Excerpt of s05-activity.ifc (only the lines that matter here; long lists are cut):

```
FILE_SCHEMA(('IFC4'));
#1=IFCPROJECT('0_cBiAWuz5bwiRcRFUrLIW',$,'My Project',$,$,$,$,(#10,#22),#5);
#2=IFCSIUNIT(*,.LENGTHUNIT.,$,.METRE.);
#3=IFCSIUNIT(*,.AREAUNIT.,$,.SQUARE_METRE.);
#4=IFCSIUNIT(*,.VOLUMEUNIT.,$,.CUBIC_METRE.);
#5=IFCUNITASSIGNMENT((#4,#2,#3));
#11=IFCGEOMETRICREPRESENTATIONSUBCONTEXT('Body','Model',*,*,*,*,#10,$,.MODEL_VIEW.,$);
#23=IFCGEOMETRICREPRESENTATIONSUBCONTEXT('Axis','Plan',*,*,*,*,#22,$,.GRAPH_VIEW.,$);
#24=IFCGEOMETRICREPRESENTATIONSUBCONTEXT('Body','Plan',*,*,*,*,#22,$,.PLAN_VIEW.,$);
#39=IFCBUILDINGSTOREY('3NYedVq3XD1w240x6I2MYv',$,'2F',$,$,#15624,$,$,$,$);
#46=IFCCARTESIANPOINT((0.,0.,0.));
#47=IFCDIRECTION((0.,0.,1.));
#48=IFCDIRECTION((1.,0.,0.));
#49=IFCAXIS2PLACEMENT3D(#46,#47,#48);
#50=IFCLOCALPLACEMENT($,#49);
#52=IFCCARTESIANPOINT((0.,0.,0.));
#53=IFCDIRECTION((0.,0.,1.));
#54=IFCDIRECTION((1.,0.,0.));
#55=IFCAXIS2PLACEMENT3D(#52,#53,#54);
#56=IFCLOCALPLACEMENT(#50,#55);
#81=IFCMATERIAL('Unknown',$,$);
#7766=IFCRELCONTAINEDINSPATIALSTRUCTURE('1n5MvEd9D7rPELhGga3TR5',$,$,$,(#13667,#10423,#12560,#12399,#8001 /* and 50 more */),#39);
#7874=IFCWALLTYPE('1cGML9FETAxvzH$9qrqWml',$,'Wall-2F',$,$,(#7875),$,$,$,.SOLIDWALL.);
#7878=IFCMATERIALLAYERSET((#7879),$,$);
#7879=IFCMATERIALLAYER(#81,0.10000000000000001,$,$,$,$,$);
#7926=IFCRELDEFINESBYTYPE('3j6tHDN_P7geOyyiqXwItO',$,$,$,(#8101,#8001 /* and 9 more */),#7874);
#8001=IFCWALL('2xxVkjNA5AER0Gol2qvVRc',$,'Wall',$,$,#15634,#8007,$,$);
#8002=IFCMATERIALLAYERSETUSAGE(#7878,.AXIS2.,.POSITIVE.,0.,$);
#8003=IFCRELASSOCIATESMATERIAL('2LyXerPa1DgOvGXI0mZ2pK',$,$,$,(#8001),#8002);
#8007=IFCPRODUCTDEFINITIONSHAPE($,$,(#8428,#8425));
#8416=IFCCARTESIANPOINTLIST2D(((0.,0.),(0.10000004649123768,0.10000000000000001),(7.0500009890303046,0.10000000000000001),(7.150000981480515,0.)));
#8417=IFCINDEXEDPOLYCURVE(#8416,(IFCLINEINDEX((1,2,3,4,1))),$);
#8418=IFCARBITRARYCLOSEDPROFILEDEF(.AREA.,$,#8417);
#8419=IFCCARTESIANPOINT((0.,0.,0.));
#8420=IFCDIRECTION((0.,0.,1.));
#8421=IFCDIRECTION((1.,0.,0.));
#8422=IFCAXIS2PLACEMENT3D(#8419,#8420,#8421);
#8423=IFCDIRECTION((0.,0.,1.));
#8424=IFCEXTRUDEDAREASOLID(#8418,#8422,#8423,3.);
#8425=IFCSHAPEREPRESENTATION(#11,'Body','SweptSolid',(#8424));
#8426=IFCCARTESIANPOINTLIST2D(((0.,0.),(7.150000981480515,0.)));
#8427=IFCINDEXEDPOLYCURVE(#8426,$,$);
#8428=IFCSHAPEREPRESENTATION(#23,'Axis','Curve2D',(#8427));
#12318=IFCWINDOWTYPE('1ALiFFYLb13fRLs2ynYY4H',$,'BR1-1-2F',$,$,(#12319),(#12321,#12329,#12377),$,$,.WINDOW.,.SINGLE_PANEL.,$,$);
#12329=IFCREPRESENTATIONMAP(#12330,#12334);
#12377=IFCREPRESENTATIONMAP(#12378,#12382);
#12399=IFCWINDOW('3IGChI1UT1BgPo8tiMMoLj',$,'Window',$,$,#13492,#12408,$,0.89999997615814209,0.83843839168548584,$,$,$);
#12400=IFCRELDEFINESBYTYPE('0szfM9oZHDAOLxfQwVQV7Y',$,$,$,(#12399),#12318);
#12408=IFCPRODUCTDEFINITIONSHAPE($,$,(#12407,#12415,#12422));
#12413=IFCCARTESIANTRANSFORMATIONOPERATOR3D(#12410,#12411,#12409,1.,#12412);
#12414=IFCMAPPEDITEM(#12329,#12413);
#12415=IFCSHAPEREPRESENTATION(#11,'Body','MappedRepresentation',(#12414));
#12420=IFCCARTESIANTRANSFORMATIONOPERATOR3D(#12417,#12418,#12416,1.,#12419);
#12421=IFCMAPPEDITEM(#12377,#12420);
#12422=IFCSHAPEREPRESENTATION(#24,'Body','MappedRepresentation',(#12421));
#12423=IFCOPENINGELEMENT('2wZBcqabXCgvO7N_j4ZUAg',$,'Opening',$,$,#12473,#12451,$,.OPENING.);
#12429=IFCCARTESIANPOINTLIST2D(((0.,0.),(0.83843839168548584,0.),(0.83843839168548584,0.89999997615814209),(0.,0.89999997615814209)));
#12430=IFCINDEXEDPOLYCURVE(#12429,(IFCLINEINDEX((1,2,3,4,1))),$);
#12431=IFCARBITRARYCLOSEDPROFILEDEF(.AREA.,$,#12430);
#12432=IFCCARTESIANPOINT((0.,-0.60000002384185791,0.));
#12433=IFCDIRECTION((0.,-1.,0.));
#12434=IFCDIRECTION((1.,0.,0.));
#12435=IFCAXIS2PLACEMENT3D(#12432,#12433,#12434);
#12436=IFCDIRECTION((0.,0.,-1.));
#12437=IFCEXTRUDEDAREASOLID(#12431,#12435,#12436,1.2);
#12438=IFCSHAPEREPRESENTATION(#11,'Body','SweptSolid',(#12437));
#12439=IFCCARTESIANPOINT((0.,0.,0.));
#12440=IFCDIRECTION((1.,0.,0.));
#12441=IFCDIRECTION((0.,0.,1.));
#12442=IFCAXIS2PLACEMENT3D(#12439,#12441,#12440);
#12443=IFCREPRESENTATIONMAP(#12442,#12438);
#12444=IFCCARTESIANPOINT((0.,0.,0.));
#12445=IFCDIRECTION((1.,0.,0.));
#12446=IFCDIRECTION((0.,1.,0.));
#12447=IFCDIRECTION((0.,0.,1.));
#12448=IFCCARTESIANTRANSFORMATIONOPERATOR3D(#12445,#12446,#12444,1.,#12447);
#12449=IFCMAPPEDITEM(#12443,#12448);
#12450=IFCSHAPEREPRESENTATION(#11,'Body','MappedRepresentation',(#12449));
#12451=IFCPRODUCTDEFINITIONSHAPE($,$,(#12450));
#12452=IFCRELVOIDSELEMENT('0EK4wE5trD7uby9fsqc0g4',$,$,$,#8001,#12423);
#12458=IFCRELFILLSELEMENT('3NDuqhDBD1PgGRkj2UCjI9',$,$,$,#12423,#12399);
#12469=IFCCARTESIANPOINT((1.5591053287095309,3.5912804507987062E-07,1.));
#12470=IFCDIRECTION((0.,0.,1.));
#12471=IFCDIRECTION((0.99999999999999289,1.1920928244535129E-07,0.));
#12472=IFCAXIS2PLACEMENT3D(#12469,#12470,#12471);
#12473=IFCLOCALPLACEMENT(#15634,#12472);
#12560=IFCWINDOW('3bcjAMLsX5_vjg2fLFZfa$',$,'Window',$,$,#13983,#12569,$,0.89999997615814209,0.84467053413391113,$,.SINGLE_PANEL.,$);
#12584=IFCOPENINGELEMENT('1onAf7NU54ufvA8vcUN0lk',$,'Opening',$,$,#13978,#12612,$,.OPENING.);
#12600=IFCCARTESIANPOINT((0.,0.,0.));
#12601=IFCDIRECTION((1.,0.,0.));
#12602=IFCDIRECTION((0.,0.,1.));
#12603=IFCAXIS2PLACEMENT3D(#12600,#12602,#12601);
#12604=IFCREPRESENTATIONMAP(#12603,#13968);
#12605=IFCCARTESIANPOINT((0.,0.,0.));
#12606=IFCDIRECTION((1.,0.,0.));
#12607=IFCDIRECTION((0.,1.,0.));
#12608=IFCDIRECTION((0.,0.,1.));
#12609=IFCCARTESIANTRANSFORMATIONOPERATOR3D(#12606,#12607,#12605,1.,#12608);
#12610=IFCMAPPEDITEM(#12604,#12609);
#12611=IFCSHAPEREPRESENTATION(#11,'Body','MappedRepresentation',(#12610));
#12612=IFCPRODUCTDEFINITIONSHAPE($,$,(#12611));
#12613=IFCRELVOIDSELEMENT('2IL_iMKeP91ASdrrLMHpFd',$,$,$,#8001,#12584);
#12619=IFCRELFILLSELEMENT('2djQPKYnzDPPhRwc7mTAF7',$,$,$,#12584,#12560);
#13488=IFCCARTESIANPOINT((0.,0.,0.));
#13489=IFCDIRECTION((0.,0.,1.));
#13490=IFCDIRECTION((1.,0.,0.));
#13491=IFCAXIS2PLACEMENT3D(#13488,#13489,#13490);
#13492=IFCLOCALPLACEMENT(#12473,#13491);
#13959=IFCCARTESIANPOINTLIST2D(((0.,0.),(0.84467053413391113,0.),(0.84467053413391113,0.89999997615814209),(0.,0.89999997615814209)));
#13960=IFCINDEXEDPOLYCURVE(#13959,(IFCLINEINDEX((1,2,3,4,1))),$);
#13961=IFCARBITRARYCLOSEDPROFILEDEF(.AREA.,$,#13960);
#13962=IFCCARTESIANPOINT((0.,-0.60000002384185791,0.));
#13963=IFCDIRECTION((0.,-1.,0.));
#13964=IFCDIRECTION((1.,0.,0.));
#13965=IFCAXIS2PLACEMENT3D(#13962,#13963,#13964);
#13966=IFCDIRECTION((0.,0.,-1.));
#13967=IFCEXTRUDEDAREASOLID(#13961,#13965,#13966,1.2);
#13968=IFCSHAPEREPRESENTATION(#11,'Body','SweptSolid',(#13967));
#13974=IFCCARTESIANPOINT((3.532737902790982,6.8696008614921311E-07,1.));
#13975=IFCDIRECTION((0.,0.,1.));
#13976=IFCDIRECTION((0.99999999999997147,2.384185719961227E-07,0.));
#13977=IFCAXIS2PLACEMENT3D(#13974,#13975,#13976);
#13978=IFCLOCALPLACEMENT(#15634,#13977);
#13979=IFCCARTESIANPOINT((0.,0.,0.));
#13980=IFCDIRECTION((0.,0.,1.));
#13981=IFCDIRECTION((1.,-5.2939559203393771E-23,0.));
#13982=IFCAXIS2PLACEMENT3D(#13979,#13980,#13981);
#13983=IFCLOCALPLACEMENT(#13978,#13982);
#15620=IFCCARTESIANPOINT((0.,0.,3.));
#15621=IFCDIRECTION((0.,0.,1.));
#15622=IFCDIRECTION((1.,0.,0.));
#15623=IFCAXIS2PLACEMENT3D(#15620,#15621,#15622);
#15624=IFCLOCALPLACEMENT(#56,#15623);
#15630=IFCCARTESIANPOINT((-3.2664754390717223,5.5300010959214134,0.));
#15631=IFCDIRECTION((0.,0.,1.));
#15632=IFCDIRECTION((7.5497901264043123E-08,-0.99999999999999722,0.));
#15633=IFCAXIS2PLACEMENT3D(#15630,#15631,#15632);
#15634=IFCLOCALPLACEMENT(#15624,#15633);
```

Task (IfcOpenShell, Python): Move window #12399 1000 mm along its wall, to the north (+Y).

```python
import ifcopenshell
import ifcopenshell.api.geometry
import ifcopenshell.util.placement
import ifcopenshell.util.unit

model = ifcopenshell.open("s05-activity.ifc")
unit_scale = ifcopenshell.util.unit.calculate_unit_scale(model)

window = model.by_guid("3IGChI1UT1BgPo8tiMMoLj")
opening = window.FillsVoids[0].RelatingOpeningElement
wall = opening.VoidsElements[0].RelatingBuildingElement

wall_matrix = ifcopenshell.util.placement.get_local_placement(wall.ObjectPlacement)
shift = wall_matrix[:3, 0] * -1 / unit_scale
before = ifcopenshell.util.placement.get_local_placement(window.ObjectPlacement)[:3, 3].copy()

# The window is placed relative to its opening, so it follows when the opening moves.
matrix = ifcopenshell.util.placement.get_local_placement(opening.ObjectPlacement)
matrix[:3, 3] += shift
ifcopenshell.api.geometry.edit_object_placement(
    model, product=opening, matrix=matrix, is_si=False, should_transform_children=True
)

after = ifcopenshell.util.placement.get_local_placement(window.ObjectPlacement)[:3, 3]
print("window moved by", (after - before).round(3) + 0.0)

model.write("s05-activity_updated.ifc")
```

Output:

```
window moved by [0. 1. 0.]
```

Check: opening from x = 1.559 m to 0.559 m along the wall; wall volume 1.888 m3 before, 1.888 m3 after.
